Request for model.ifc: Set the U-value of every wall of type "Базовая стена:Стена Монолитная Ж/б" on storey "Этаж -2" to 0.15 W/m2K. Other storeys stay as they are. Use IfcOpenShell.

First a look at what the model holds.

```python
import ifcopenshell
import ifcopenshell.util.element

model = ifcopenshell.open("model.ifc")
print(model.schema)
storey = next(s for s in model.by_type("IfcBuildingStorey") if s.Name == "Этаж -2")
walls = [e for e in ifcopenshell.util.element.get_decomposition(storey) if e.is_a("IfcWall")]
seen = {}
for e in walls:
    element_type = ifcopenshell.util.element.get_type(e)
    key = (element_type.Name if element_type != e and element_type else None, ifcopenshell.util.element.get_pset(e, "Pset_WallCommon", "ThermalTransmittance"))
    seen[key] = seen.get(key, 0) + 1
for (name, value), count in sorted(seen.items(), key=str):
    print(count, "x", name, "|", value)
```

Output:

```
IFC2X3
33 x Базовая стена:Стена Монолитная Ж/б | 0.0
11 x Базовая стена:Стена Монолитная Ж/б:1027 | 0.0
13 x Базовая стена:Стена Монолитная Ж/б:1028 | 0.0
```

```python
import ifcopenshell
import ifcopenshell.api.pset
import ifcopenshell.util.element

model = ifcopenshell.open("model.ifc")

storey = next(s for s in model.by_type("IfcBuildingStorey") if s.Name == "Этаж -2")
walls = [e for e in ifcopenshell.util.element.get_decomposition(storey) if e.is_a("IfcWall")]

count = 0
for e in walls:
    element_type = ifcopenshell.util.element.get_type(e)
    if element_type in (None, e) or element_type.Name != "Базовая стена:Стена Монолитная Ж/б":
        continue
    # add_pset returns the element's existing set when there is one.
    pset = ifcopenshell.api.pset.add_pset(model, product=e, name="Pset_WallCommon")
    ifcopenshell.api.pset.edit_pset(model, pset=pset, properties={"ThermalTransmittance": 0.15})
    count += 1

print(count, "walls updated")

model.write("model_v2.ifc")
```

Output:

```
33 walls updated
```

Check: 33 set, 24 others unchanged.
